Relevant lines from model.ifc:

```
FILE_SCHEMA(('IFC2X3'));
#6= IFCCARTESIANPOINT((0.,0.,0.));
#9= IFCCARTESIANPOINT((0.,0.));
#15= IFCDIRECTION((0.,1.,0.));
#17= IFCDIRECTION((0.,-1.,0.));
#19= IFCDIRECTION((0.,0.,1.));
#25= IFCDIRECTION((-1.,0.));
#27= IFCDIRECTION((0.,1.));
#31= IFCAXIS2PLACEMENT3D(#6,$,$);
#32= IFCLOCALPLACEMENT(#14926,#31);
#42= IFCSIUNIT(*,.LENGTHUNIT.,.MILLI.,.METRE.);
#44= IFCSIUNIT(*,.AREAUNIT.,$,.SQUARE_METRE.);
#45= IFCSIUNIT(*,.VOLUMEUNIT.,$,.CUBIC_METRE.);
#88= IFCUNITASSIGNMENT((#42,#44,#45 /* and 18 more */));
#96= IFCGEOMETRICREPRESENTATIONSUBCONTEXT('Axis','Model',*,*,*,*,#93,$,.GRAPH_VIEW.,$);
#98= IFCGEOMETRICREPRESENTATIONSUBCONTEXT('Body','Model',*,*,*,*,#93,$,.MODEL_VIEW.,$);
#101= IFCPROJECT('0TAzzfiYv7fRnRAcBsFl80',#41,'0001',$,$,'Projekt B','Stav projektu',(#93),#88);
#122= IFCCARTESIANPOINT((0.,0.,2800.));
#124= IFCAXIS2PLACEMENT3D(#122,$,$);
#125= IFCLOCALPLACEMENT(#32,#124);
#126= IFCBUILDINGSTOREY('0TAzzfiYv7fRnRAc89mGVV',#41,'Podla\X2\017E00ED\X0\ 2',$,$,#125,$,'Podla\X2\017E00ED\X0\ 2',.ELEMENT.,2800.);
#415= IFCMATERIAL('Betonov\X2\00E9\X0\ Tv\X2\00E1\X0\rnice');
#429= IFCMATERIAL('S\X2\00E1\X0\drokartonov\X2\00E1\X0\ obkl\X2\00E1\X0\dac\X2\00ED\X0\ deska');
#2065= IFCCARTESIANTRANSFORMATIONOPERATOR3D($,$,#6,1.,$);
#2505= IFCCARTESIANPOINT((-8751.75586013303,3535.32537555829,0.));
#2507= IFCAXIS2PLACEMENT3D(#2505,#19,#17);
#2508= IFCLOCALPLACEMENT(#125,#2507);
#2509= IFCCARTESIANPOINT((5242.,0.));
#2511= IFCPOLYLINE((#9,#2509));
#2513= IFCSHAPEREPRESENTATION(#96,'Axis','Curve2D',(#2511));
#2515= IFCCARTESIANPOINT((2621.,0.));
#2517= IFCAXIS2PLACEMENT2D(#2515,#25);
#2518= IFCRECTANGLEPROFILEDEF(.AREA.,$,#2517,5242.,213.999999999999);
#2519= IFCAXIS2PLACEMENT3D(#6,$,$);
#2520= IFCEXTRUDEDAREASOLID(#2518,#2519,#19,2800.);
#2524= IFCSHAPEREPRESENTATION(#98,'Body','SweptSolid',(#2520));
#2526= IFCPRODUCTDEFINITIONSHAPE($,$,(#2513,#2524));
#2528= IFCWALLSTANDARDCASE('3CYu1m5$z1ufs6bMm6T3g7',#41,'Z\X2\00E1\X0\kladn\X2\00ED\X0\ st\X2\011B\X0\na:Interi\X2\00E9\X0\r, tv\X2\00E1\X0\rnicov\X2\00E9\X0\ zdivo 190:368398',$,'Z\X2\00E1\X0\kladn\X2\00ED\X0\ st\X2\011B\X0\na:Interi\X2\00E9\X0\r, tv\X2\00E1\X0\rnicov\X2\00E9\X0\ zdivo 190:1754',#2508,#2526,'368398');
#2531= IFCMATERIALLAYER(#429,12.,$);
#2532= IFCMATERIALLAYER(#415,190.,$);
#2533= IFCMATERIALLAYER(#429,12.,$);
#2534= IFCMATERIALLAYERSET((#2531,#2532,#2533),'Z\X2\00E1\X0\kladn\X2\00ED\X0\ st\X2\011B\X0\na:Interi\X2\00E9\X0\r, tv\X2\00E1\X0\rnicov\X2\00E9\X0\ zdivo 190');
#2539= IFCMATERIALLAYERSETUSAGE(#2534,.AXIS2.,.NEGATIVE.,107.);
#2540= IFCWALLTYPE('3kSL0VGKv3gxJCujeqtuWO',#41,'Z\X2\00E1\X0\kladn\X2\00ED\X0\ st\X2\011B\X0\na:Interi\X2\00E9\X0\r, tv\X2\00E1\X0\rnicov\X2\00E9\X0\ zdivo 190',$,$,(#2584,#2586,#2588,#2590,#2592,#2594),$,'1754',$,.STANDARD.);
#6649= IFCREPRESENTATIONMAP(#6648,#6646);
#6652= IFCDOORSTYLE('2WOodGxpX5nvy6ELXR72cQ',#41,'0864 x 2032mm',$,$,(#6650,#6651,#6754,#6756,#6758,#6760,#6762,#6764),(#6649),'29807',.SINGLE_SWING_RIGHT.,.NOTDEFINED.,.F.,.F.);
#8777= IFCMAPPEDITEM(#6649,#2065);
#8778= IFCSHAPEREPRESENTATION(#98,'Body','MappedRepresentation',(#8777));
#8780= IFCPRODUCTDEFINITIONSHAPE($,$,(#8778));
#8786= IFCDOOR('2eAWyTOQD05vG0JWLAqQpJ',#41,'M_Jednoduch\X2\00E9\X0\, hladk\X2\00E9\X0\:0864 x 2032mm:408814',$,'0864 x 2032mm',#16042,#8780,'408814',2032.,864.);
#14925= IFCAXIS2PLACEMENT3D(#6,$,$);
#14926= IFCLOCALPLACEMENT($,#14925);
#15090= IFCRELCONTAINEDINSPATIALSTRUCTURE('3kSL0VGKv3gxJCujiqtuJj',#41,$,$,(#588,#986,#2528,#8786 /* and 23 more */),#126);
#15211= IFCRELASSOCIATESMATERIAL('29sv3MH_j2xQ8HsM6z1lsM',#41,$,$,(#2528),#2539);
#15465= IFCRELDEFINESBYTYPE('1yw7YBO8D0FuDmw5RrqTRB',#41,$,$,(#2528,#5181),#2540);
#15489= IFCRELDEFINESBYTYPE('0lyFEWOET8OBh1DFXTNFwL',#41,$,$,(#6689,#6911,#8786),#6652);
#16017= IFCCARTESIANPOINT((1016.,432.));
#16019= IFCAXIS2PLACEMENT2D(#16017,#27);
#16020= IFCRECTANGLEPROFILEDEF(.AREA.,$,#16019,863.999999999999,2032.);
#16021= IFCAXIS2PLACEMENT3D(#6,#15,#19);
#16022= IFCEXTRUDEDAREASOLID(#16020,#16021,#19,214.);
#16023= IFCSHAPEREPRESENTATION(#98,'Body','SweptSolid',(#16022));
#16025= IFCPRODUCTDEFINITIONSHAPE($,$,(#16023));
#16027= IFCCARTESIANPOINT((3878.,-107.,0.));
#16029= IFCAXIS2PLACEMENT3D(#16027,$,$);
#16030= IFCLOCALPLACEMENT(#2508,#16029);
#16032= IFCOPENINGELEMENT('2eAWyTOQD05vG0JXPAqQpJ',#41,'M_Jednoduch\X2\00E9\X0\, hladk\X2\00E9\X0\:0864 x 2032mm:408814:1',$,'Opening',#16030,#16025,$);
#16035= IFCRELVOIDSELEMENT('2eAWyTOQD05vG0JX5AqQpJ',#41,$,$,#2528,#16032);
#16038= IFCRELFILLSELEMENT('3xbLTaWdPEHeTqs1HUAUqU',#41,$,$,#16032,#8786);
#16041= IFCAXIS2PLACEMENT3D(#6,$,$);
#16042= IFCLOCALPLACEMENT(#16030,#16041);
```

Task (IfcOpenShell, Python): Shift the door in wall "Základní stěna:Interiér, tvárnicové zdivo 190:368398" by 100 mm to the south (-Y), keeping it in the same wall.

```python
import ifcopenshell
import ifcopenshell.api.geometry
import ifcopenshell.util.placement

model = ifcopenshell.open("model.ifc")

door = model.by_guid("2eAWyTOQD05vG0JWLAqQpJ")
opening = door.FillsVoids[0].RelatingOpeningElement
wall = opening.VoidsElements[0].RelatingBuildingElement

wall_matrix = ifcopenshell.util.placement.get_local_placement(wall.ObjectPlacement)
shift = wall_matrix[:3, 0] * 100.0
before = ifcopenshell.util.placement.get_local_placement(door.ObjectPlacement)[:3, 3].copy()

# The door is placed relative to its opening, so it follows when the opening moves.
matrix = ifcopenshell.util.placement.get_local_placement(opening.ObjectPlacement)
matrix[:3, 3] += shift
ifcopenshell.api.geometry.edit_object_placement(
    model, product=opening, matrix=matrix, is_si=False, should_transform_children=True
)

after = ifcopenshell.util.placement.get_local_placement(door.ObjectPlacement)[:3, 3]
print("door moved by", (after - before).round(3) + 0.0)

model.write("model_v2.ifc")
```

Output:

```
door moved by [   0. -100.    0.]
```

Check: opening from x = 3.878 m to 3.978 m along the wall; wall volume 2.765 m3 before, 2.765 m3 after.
